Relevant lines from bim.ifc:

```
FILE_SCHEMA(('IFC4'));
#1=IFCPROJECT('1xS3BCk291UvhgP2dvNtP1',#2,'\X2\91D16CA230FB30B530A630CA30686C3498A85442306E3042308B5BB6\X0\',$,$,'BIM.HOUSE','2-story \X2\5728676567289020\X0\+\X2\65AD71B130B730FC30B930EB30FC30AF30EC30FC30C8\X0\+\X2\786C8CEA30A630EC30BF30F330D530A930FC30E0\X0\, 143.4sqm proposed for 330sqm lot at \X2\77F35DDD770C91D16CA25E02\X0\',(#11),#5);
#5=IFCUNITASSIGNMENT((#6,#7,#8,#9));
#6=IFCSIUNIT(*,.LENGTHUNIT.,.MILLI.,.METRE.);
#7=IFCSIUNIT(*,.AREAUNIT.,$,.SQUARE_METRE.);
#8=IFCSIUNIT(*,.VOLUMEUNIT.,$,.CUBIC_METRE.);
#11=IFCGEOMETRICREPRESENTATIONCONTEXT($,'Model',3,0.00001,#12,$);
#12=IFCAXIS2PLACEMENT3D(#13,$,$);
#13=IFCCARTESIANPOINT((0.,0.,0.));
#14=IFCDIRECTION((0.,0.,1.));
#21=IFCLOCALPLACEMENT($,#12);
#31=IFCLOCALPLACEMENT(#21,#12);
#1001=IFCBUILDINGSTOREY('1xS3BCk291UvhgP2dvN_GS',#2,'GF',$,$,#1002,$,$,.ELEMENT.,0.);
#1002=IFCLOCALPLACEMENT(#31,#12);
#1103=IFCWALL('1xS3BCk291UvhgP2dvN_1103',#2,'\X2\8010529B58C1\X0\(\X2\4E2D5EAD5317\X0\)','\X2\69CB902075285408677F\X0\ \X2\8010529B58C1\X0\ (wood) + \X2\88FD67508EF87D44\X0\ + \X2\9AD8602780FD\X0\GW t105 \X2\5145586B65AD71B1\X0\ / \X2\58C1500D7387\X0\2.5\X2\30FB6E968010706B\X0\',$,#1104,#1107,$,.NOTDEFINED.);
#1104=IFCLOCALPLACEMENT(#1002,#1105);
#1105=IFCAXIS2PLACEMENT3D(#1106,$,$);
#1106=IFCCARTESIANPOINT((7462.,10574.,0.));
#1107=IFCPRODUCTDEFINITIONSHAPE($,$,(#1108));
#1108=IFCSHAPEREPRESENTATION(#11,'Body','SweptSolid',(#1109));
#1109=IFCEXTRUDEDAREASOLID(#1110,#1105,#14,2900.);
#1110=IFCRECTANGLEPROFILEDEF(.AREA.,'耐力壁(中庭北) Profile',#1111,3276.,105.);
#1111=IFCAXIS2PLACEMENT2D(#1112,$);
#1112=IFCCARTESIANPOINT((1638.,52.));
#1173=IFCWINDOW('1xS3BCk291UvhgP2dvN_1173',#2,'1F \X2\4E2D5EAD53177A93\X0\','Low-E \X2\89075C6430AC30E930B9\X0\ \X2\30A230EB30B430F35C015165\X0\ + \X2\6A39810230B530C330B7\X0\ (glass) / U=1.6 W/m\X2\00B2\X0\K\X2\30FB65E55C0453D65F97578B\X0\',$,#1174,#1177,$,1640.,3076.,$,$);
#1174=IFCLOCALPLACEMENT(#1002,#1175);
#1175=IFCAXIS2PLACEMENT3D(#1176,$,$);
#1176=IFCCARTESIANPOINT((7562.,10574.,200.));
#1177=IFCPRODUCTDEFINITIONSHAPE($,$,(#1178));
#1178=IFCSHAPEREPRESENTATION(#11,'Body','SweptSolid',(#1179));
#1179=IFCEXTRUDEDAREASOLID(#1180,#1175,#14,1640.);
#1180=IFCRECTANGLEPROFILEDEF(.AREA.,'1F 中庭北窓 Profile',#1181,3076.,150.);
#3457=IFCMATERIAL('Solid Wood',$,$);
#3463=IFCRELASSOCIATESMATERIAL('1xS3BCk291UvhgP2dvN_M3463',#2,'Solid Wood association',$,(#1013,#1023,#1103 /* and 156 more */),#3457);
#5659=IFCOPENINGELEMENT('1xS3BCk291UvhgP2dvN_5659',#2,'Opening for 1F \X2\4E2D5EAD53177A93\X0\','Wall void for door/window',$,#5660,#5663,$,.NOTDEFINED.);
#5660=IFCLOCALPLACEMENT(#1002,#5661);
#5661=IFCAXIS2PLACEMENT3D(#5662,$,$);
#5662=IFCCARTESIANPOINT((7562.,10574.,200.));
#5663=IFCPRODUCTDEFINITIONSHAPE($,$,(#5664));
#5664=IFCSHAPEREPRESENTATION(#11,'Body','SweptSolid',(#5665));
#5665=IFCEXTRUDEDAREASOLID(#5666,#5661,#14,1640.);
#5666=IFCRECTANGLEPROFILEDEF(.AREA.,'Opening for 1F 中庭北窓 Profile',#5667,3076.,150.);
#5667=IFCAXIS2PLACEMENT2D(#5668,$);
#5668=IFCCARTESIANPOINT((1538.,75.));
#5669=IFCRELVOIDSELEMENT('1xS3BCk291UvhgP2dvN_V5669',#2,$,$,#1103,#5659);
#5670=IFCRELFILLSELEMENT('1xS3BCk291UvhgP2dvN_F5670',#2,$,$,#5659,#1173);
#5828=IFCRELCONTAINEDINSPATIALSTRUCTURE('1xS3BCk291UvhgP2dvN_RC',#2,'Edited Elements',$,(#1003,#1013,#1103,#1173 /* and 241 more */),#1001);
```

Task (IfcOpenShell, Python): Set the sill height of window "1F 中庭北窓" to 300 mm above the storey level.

```python
import numpy as np
import ifcopenshell
import ifcopenshell.api.geometry
import ifcopenshell.geom
import ifcopenshell.util.element
import ifcopenshell.util.placement
import ifcopenshell.util.shape
import ifcopenshell.util.unit

model = ifcopenshell.open("bim.ifc")
unit_scale = ifcopenshell.util.unit.calculate_unit_scale(model)

window = model.by_guid("1xS3BCk291UvhgP2dvN_1173")
opening = window.FillsVoids[0].RelatingOpeningElement
storey = ifcopenshell.util.element.get_container(window, ifc_class="IfcBuildingStorey")
level = ifcopenshell.util.placement.get_local_placement(storey.ObjectPlacement)[2, 3]

# The opening's origin need not be at the sill, so measure its lowest point.
shape = ifcopenshell.geom.create_shape(ifcopenshell.geom.settings(), opening)
bottom = ifcopenshell.util.shape.get_shape_bottom_elevation(shape, shape.geometry) / unit_scale
dz = level + 0.3 / unit_scale - bottom

shift = np.array([0.0, 0.0, dz])
# The window is not placed relative to its opening, so move both.
for product in (opening, window):
    matrix = ifcopenshell.util.placement.get_local_placement(product.ObjectPlacement)
    matrix[:3, 3] += shift
    ifcopenshell.api.geometry.edit_object_placement(model, product=product, matrix=matrix, is_si=False)

print(f"moved by {dz * unit_scale:+.3f} m")

model.write("bim_updated.ifc")
```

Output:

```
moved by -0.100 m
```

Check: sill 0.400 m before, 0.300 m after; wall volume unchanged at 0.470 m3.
